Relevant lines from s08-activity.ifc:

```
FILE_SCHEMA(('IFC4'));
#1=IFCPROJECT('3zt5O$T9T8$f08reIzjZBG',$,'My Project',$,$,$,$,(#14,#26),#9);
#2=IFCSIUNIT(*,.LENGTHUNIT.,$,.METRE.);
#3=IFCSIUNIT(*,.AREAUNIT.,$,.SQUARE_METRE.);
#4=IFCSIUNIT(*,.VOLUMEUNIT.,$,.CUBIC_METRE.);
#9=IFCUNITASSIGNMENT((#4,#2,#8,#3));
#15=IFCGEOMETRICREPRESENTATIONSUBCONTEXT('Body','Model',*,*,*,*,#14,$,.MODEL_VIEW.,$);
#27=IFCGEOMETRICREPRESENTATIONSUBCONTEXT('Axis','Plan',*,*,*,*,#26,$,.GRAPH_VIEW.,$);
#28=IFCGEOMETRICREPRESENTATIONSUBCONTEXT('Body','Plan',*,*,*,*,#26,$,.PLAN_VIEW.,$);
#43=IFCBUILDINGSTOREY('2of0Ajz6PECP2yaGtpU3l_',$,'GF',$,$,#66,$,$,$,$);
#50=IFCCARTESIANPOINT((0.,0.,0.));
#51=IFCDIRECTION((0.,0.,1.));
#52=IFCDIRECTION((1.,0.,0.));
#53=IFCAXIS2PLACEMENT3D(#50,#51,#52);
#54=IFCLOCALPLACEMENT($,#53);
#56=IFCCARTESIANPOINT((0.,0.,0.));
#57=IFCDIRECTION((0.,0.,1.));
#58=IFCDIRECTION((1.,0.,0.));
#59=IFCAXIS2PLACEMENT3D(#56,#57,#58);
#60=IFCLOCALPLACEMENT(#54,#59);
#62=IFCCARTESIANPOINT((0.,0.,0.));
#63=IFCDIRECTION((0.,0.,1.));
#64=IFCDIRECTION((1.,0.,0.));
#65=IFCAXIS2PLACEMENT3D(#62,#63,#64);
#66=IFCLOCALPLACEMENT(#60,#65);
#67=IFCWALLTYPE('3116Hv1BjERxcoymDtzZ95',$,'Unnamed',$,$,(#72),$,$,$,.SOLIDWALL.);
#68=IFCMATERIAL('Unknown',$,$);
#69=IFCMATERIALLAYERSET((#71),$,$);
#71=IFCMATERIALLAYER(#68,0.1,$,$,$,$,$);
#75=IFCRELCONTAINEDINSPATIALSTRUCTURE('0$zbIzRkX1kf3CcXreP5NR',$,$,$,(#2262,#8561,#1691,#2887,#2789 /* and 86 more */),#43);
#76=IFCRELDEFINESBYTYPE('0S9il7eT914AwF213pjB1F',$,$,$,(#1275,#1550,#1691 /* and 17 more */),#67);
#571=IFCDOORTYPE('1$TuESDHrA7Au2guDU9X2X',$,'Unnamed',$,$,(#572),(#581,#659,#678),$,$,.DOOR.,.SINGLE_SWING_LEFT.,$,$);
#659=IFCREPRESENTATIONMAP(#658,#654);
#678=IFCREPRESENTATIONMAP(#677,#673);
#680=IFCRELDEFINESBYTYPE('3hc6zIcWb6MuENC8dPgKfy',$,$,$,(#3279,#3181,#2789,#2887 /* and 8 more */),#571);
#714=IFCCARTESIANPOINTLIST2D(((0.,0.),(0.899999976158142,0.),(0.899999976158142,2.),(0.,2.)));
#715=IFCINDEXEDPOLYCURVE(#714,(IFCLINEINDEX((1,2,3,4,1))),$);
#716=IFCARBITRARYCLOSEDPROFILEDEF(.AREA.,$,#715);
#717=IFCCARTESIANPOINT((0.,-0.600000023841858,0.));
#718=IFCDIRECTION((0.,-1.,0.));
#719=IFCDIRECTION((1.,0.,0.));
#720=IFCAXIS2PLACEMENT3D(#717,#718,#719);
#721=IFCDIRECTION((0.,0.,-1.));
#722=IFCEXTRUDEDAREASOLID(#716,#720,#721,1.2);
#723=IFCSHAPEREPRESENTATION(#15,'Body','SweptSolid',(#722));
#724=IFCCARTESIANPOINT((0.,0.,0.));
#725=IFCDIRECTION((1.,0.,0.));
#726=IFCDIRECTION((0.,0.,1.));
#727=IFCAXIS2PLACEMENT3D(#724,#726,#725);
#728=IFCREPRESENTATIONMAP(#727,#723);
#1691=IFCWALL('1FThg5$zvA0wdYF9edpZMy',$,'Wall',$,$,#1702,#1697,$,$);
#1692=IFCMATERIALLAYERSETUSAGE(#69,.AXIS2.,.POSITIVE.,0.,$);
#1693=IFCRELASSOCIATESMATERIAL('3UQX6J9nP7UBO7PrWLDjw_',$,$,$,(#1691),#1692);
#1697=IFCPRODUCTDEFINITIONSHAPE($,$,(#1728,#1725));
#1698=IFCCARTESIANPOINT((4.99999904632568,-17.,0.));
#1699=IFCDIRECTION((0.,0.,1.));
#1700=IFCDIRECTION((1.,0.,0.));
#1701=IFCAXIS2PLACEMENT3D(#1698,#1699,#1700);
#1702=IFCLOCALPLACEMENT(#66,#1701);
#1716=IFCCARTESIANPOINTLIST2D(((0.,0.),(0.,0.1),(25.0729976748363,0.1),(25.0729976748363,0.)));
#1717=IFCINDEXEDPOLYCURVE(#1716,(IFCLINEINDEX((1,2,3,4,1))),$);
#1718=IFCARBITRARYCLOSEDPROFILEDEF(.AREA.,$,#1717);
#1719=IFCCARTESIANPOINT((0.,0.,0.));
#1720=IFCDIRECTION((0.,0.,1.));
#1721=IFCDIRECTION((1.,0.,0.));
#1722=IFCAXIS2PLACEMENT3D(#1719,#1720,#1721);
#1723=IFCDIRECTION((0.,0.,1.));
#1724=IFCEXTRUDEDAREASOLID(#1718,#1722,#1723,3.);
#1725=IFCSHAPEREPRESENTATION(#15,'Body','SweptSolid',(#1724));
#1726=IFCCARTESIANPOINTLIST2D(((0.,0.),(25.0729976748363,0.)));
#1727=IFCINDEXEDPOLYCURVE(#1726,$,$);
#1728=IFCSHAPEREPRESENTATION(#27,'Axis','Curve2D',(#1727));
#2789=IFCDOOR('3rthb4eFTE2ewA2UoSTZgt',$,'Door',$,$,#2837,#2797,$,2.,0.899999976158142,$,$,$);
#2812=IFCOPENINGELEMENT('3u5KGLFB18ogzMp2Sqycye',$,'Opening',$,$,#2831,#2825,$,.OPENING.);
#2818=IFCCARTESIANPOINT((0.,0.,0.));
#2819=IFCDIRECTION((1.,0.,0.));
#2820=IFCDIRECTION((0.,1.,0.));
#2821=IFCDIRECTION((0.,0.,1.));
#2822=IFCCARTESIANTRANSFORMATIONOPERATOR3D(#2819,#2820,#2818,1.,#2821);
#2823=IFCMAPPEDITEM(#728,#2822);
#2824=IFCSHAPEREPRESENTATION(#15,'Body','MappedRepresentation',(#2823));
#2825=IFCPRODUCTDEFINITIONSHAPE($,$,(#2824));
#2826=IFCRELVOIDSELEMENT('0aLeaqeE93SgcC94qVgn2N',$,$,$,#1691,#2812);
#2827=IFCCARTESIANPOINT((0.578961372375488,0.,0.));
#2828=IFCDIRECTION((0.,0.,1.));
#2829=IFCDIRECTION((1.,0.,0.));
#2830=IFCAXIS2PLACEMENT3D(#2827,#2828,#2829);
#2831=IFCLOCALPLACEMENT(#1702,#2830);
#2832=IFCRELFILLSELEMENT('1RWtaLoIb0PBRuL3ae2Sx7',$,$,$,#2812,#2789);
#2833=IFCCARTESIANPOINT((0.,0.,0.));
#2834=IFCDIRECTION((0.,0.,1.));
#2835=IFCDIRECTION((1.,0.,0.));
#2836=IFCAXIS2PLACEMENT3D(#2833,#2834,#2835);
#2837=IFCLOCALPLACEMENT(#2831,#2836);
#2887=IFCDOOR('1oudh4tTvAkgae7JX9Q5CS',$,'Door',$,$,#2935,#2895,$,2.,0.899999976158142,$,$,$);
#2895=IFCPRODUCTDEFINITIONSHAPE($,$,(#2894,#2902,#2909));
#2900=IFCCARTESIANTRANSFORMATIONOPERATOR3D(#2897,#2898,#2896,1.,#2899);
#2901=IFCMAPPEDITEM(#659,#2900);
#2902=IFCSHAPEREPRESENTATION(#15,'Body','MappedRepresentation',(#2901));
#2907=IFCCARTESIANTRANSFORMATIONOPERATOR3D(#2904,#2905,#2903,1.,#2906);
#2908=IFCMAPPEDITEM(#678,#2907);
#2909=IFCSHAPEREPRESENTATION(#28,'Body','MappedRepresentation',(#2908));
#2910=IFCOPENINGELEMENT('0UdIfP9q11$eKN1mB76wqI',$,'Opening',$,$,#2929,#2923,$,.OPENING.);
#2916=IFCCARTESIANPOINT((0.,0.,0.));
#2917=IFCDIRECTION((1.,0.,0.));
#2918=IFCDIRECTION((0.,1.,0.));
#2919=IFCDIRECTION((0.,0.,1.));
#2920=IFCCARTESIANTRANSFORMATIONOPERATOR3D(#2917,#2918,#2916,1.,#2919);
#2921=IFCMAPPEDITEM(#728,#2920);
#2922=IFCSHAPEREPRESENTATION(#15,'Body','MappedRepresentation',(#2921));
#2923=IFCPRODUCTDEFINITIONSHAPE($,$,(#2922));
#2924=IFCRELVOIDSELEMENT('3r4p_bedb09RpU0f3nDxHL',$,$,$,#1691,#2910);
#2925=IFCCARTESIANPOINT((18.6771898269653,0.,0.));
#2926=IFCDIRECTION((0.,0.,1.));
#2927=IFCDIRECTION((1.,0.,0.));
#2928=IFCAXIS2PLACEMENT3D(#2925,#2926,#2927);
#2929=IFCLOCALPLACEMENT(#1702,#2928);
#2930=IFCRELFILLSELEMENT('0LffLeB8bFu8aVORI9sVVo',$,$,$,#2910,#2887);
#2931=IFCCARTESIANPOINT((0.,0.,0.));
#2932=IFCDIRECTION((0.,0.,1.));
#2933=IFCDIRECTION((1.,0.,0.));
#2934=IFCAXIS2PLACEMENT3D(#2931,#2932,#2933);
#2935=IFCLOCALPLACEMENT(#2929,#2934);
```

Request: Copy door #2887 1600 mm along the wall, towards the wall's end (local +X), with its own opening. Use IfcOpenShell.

```python
import ifcopenshell
import ifcopenshell.api.feature
import ifcopenshell.api.geometry
import ifcopenshell.api.root
import ifcopenshell.geom
import ifcopenshell.util.element
import ifcopenshell.util.placement
import ifcopenshell.util.shape

model = ifcopenshell.open("s08-activity.ifc")
settings = ifcopenshell.geom.settings()


def volume(element):
    """Net volume in cubic metres, openings subtracted."""
    shape = ifcopenshell.geom.create_shape(settings, element)
    return ifcopenshell.util.shape.get_volume(shape.geometry)


door = model.by_guid("1oudh4tTvAkgae7JX9Q5CS")
opening = door.FillsVoids[0].RelatingOpeningElement
wall = opening.VoidsElements[0].RelatingBuildingElement
before = volume(wall)
shift = ifcopenshell.util.placement.get_local_placement(wall.ObjectPlacement)[:3, 0] * 1.6

# copy_class copies the void relationship, type, container and properties, but no geometry.
new_opening = ifcopenshell.api.root.copy_class(model, product=opening)
new_opening.Representation = ifcopenshell.util.element.copy_deep(
    model, opening.Representation, exclude=["IfcGeometricRepresentationContext", "IfcRepresentationMap"]
)
new_door = ifcopenshell.api.root.copy_class(model, product=door)
new_door.Representation = ifcopenshell.util.element.copy_deep(
    model, door.Representation, exclude=["IfcGeometricRepresentationContext", "IfcRepresentationMap"]
)
ifcopenshell.api.feature.add_filling(model, opening=new_opening, element=new_door)

for old, new in ((opening, new_opening), (door, new_door)):
    matrix = ifcopenshell.util.placement.get_local_placement(old.ObjectPlacement)
    matrix[:3, 3] += shift
    ifcopenshell.api.geometry.edit_object_placement(model, product=new, matrix=matrix, is_si=False)

after = volume(wall)

print(f"wall volume {before:.3f} -> {after:.3f} m3")

model.write("s08-activity_rev.ifc")
```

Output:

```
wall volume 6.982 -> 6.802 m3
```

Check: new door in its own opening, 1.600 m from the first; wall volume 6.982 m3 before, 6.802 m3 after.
